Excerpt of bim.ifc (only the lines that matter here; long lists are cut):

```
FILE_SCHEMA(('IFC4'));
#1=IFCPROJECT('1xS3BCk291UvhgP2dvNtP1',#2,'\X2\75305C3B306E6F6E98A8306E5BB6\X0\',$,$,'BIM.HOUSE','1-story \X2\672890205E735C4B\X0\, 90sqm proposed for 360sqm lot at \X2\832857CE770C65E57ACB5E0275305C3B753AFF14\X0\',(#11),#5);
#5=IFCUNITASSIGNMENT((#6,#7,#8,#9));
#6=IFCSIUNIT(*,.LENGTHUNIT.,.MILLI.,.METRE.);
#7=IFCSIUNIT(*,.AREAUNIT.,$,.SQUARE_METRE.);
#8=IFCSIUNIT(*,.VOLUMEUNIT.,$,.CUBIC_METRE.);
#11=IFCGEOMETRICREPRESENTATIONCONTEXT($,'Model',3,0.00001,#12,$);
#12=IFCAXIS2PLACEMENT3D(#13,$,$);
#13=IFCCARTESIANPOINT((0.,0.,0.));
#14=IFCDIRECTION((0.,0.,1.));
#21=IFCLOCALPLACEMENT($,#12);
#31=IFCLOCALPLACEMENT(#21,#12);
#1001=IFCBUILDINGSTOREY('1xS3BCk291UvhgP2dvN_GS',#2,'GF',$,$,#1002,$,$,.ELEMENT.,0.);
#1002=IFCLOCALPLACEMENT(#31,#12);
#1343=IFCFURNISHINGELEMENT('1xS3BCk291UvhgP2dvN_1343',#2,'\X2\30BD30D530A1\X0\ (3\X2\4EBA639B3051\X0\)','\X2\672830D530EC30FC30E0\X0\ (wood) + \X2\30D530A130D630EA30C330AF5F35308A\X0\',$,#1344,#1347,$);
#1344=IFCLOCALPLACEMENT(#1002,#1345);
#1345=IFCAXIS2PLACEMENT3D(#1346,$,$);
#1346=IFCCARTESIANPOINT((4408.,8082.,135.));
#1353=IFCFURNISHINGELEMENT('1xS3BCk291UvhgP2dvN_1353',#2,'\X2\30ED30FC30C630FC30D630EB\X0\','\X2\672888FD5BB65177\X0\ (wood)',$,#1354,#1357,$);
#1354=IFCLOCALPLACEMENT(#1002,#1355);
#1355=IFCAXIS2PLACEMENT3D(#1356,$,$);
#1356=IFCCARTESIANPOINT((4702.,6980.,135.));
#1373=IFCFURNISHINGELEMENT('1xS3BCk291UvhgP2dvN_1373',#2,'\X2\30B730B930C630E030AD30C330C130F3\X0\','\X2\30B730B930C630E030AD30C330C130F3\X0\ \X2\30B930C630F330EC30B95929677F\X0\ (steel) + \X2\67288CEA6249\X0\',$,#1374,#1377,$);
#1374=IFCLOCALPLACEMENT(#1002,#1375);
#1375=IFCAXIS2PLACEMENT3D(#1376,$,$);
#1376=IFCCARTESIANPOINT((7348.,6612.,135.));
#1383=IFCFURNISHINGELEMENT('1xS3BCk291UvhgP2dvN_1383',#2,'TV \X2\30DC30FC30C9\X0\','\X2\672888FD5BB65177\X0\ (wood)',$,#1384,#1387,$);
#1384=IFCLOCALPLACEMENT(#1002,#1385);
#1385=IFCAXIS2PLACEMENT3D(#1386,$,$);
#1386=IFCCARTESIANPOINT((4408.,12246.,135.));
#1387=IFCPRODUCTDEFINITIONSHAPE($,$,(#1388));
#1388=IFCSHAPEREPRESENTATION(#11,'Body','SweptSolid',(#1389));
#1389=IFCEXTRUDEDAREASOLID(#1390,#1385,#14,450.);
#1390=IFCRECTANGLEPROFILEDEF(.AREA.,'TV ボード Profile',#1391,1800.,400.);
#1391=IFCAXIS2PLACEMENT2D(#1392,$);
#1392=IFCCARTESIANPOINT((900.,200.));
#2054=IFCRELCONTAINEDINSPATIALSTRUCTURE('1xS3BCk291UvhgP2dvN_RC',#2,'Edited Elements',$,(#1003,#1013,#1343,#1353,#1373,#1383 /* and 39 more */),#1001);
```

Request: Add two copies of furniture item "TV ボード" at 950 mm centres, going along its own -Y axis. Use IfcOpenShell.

```python
import ifcopenshell
import ifcopenshell.api.geometry
import ifcopenshell.api.root
import ifcopenshell.util.element
import ifcopenshell.util.placement
import ifcopenshell.util.unit

model = ifcopenshell.open("bim.ifc")
unit_scale = ifcopenshell.util.unit.calculate_unit_scale(model)


def reuse_history(source, copy):
    """copy_class also copies each property set's owner history, people and application; keep the originals."""
    for rel in copy.IsDefinedBy:
        if rel.is_a("IfcRelDefinesByProperties") and (history := rel.RelatingPropertyDefinition.OwnerHistory):
            rel.RelatingPropertyDefinition.OwnerHistory = source.OwnerHistory
            ifcopenshell.util.element.remove_deep2(model, history)


source = model.by_id(1383)
base = ifcopenshell.util.placement.get_local_placement(source.ObjectPlacement)
step = -base[:3, 1] * 0.95 / unit_scale

for i in range(1, 3):
    copy = ifcopenshell.api.root.copy_class(model, product=source)
    copy.Representation = ifcopenshell.util.element.copy_deep(
        model, source.Representation, exclude=["IfcGeometricRepresentationContext", "IfcRepresentationMap"]
    )
    reuse_history(source, copy)
    matrix = base.copy()
    matrix[:3, 3] += i * step
    print("added at", matrix[:3, 3].round(3) + 0.0)
    ifcopenshell.api.geometry.edit_object_placement(model, product=copy, matrix=matrix, is_si=False)

model.write("bim_v2.ifc")
```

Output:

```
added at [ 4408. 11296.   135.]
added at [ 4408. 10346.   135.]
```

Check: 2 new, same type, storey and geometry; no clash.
